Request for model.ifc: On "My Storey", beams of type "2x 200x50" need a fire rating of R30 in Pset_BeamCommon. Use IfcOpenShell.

First a look at what the model holds.

```python
import ifcopenshell
import ifcopenshell.util.element

model = ifcopenshell.open("model.ifc")
print(model.schema)
storey = next(s for s in model.by_type("IfcBuildingStorey") if s.Name == "My Storey")
beams = [e for e in ifcopenshell.util.element.get_decomposition(storey) if e.is_a("IfcBeam")]
seen = {}
for e in beams:
    element_type = ifcopenshell.util.element.get_type(e)
    key = (element_type.Name if element_type != e and element_type else None, ifcopenshell.util.element.get_pset(e, "Pset_BeamCommon", "FireRating"))
    seen[key] = seen.get(key, 0) + 1
for (name, value), count in sorted(seen.items(), key=str):
    print(count, "x", name, "|", value)
```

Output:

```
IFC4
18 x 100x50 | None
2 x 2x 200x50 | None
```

```python
import ifcopenshell
import ifcopenshell.api.pset
import ifcopenshell.util.element

model = ifcopenshell.open("model.ifc")

storey = next(s for s in model.by_type("IfcBuildingStorey") if s.Name == "My Storey")
beams = [e for e in ifcopenshell.util.element.get_decomposition(storey) if e.is_a("IfcBeam")]

count = 0
for e in beams:
    element_type = ifcopenshell.util.element.get_type(e)
    if element_type in (None, e) or element_type.Name != "2x 200x50":
        continue
    # add_pset returns the element's existing set when there is one.
    pset = ifcopenshell.api.pset.add_pset(model, product=e, name="Pset_BeamCommon")
    ifcopenshell.api.pset.edit_pset(model, pset=pset, properties={"FireRating": "R30"})
    count += 1

print(count, "beams updated")

model.write("model_updated.ifc")
```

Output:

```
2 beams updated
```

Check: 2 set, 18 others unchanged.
